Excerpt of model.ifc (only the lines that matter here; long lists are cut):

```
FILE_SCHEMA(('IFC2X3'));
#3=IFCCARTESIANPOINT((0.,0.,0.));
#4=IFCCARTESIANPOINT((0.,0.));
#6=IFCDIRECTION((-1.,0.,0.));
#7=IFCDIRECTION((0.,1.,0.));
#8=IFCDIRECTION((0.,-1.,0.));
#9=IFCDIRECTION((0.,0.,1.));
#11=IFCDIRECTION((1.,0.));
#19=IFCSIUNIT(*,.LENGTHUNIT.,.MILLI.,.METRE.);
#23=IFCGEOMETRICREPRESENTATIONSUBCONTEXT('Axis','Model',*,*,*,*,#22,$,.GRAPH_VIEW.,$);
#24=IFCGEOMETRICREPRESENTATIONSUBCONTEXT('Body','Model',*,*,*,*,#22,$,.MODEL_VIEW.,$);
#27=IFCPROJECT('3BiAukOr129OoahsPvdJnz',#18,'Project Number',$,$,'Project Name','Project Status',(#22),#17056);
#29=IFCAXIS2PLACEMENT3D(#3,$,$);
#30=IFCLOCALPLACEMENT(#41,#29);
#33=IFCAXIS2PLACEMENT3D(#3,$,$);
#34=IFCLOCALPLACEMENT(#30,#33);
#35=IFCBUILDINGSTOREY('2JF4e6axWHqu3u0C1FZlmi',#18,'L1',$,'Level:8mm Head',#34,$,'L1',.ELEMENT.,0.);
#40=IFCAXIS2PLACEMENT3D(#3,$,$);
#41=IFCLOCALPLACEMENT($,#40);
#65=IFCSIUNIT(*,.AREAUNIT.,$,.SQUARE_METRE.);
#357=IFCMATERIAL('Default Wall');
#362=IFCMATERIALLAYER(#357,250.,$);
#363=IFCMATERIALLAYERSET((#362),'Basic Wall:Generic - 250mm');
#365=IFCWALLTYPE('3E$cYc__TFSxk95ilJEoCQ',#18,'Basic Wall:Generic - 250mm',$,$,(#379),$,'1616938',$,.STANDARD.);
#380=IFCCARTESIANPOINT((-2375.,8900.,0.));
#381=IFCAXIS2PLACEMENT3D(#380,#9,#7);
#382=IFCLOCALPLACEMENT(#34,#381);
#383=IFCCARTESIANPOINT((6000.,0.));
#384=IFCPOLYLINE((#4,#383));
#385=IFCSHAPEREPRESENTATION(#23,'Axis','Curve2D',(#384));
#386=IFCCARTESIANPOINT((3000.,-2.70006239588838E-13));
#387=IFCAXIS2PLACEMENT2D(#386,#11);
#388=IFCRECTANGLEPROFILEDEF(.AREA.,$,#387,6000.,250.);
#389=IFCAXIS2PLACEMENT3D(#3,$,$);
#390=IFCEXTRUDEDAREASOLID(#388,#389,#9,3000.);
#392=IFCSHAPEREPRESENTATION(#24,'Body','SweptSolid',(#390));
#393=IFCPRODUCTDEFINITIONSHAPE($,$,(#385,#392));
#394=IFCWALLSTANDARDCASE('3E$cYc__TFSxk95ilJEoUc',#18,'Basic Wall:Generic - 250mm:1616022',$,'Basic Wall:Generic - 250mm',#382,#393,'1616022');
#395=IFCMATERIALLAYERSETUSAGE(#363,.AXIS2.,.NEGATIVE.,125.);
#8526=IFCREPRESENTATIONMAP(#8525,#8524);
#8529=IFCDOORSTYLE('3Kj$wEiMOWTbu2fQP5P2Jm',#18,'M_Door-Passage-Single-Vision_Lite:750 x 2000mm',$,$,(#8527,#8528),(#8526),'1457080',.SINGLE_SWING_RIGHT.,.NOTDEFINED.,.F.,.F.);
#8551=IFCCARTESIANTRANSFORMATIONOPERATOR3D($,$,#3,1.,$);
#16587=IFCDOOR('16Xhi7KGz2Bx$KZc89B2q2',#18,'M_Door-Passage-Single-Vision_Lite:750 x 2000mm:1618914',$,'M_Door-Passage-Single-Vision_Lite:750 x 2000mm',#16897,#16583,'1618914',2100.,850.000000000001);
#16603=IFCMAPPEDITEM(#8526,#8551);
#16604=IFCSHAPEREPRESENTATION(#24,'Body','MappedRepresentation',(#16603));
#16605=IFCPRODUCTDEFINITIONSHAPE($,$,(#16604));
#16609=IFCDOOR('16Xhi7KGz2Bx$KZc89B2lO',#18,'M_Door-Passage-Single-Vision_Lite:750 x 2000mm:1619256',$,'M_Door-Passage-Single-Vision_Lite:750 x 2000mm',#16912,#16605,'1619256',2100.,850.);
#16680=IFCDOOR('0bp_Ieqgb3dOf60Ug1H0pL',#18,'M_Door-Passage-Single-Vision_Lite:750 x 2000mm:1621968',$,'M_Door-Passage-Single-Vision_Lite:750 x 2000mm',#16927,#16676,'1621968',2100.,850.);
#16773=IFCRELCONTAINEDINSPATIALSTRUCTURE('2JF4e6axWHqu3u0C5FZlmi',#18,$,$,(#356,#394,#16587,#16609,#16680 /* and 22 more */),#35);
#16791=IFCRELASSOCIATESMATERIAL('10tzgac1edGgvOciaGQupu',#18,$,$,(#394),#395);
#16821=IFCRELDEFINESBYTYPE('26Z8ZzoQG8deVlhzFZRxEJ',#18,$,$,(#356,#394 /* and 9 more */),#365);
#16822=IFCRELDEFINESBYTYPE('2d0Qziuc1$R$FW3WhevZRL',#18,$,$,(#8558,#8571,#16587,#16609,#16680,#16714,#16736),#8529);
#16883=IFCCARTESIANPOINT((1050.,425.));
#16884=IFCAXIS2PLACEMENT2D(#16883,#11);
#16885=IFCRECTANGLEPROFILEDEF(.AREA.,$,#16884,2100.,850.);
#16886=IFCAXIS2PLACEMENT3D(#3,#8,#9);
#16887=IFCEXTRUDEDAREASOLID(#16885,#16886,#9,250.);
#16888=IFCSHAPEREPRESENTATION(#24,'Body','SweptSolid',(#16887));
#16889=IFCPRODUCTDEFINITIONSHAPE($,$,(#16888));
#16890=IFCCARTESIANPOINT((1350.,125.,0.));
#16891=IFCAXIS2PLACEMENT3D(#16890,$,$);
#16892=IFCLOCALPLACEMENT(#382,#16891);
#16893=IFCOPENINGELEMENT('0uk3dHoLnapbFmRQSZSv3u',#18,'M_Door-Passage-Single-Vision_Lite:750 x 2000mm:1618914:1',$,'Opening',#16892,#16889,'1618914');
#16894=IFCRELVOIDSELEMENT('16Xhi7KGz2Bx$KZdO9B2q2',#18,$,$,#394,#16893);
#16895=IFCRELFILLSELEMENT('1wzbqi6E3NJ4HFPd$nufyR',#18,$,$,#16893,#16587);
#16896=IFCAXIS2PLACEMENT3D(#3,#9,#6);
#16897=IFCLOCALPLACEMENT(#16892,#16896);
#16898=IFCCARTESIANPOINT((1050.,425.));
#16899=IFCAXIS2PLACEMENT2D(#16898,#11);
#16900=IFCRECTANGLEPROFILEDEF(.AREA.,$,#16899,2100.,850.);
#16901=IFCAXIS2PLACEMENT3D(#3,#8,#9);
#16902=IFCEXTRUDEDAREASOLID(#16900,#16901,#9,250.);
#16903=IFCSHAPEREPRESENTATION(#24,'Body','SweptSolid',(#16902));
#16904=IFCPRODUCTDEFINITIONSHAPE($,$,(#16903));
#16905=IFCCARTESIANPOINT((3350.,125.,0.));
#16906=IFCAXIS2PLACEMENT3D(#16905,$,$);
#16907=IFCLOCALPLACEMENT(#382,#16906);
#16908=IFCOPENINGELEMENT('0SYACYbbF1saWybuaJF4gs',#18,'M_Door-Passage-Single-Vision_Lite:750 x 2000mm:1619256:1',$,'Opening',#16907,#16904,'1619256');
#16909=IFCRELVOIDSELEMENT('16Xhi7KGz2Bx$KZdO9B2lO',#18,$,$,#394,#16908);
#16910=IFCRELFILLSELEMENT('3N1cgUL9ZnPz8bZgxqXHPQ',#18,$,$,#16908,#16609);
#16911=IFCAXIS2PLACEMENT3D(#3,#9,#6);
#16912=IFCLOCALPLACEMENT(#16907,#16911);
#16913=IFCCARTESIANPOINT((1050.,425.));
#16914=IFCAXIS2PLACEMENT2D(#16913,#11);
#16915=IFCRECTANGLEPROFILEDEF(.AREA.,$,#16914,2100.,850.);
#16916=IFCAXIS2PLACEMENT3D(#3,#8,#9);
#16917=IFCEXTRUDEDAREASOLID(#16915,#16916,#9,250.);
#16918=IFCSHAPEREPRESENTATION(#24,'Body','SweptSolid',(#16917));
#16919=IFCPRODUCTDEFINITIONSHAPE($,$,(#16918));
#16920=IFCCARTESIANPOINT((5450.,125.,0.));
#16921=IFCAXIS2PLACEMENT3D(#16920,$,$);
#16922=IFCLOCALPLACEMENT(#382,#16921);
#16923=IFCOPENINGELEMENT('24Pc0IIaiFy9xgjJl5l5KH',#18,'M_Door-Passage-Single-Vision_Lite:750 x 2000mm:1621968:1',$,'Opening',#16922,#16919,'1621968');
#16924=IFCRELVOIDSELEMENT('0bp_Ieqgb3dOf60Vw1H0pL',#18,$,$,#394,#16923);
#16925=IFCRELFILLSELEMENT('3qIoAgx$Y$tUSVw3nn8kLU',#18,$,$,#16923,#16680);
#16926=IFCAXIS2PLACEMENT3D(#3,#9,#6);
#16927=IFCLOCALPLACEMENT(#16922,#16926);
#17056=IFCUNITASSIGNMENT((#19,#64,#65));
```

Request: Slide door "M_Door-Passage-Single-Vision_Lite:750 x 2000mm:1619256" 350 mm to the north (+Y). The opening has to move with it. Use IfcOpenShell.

```python
import ifcopenshell
import ifcopenshell.api.geometry
import ifcopenshell.util.placement
import ifcopenshell.util.unit

model = ifcopenshell.open("model.ifc")
unit_scale = ifcopenshell.util.unit.calculate_unit_scale(model)

door = model.by_guid("16Xhi7KGz2Bx$KZc89B2lO")
opening = door.FillsVoids[0].RelatingOpeningElement
wall = opening.VoidsElements[0].RelatingBuildingElement

wall_matrix = ifcopenshell.util.placement.get_local_placement(wall.ObjectPlacement)
shift = wall_matrix[:3, 0] * 0.35 / unit_scale
before = ifcopenshell.util.placement.get_local_placement(door.ObjectPlacement)[:3, 3].copy()

# The door is placed relative to its opening, so it follows when the opening moves.
matrix = ifcopenshell.util.placement.get_local_placement(opening.ObjectPlacement)
matrix[:3, 3] += shift
ifcopenshell.api.geometry.edit_object_placement(
    model, product=opening, matrix=matrix, is_si=False, should_transform_children=True
)

after = ifcopenshell.util.placement.get_local_placement(door.ObjectPlacement)[:3, 3]
print("door moved by", (after - before).round(3) + 0.0)

model.write("model_updated.ifc")
```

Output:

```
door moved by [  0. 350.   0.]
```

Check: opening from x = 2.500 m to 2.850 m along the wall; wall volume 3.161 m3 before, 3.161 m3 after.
